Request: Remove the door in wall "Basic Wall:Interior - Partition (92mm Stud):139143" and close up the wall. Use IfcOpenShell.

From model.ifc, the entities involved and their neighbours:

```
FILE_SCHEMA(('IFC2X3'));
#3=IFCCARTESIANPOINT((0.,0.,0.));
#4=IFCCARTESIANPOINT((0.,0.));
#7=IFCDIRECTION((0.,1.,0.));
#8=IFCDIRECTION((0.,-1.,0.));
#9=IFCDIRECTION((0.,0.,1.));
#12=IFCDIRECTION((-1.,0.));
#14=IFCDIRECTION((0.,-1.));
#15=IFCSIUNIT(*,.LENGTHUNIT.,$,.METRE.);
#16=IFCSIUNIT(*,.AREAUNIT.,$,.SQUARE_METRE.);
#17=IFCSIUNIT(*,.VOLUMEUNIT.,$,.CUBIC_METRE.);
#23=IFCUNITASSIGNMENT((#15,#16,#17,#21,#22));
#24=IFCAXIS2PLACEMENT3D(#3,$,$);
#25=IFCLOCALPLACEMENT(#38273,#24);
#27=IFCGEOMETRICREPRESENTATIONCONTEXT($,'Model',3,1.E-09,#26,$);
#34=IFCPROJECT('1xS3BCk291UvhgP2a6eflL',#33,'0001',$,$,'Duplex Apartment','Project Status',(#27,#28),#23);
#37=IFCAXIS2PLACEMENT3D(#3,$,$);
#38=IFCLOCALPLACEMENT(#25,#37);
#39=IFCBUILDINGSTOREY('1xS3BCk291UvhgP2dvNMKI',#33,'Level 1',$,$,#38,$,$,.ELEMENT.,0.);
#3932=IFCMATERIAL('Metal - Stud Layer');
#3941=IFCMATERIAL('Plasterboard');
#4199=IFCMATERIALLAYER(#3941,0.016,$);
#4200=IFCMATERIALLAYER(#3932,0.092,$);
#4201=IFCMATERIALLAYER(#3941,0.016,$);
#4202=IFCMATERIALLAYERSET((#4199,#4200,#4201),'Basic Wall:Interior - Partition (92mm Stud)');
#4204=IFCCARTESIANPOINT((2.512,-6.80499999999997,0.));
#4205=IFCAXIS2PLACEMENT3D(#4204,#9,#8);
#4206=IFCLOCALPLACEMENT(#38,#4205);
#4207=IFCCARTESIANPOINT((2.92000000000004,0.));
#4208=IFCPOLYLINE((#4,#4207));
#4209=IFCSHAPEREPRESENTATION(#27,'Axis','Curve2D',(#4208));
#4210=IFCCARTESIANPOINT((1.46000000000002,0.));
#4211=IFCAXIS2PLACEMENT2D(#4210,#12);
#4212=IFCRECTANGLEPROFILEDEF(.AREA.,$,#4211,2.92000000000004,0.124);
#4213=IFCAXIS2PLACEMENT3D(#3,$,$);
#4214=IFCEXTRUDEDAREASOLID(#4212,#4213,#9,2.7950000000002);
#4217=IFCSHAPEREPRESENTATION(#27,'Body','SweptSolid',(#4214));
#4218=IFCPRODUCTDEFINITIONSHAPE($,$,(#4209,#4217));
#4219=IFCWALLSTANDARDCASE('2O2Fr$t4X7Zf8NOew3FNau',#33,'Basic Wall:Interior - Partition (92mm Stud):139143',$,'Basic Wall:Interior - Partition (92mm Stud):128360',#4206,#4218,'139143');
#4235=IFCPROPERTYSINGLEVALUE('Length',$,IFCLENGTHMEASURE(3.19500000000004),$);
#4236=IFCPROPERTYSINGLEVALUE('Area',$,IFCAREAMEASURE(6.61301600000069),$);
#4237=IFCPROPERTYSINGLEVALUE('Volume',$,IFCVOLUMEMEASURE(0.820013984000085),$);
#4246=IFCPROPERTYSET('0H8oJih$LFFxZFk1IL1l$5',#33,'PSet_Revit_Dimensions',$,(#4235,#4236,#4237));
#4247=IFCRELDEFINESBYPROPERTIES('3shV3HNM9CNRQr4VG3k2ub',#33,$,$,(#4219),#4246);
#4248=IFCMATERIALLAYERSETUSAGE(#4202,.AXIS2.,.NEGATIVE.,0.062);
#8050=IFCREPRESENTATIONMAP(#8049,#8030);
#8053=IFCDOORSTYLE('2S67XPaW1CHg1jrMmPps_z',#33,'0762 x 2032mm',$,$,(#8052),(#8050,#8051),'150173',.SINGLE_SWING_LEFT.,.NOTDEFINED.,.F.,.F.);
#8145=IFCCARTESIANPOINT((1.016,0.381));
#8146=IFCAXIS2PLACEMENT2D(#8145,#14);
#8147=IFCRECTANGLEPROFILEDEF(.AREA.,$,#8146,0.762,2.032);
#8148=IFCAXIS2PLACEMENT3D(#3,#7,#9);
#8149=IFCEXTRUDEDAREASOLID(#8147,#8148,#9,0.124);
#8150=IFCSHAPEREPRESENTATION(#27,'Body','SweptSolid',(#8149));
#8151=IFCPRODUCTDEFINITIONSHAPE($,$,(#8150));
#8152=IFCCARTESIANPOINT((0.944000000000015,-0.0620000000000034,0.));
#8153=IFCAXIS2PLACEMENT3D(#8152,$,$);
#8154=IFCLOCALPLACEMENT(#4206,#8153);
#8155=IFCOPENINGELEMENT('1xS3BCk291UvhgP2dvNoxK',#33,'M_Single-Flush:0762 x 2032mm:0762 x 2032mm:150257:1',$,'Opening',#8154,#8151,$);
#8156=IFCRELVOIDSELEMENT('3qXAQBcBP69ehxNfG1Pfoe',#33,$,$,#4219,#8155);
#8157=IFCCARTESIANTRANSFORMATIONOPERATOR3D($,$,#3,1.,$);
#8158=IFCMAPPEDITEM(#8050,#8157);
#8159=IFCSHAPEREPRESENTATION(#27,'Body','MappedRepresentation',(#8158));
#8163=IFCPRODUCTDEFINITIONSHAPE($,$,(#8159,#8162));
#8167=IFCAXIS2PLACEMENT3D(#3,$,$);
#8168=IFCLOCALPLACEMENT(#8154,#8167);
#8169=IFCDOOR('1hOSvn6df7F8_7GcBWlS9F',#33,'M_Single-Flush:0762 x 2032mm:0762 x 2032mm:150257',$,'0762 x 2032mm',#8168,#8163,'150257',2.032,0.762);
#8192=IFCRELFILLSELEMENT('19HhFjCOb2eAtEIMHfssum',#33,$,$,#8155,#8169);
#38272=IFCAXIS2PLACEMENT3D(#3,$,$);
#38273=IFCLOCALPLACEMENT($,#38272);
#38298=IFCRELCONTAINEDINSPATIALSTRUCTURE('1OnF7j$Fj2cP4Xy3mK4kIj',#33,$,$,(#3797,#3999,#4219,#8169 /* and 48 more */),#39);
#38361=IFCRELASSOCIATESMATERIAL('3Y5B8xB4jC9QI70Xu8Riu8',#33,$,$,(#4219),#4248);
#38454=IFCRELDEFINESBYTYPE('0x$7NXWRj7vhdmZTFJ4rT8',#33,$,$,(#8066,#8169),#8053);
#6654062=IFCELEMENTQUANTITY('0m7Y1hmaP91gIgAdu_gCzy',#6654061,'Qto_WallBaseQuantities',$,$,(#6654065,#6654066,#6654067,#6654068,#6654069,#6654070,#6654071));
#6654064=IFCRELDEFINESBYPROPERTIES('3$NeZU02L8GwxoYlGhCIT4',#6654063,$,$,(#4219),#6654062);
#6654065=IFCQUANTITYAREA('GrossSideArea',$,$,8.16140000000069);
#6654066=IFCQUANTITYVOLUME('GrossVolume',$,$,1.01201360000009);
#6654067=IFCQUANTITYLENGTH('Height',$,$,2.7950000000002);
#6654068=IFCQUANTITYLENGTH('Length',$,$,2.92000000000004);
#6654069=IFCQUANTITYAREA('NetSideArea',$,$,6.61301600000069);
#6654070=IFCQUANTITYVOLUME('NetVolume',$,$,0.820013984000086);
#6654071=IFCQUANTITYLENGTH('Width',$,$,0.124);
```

```python
import ifcopenshell
import ifcopenshell.api.feature
import ifcopenshell.api.pset
import ifcopenshell.api.root
import ifcopenshell.geom
import ifcopenshell.util.element
import ifcopenshell.util.shape
import ifcopenshell.util.unit

model = ifcopenshell.open("model.ifc")
area_scale = ifcopenshell.util.unit.calculate_unit_scale(model, "AREAUNIT")
volume_scale = ifcopenshell.util.unit.calculate_unit_scale(model, "VOLUMEUNIT")
settings = ifcopenshell.geom.settings()


def volume(element):
    """Net volume in cubic metres, openings subtracted."""
    shape = ifcopenshell.geom.create_shape(settings, element)
    return ifcopenshell.util.shape.get_volume(shape.geometry)


door = model.by_id(8169)
opening = door.FillsVoids[0].RelatingOpeningElement
wall = opening.VoidsElements[0].RelatingBuildingElement
before = volume(wall)

ifcopenshell.api.root.remove_product(model, product=door)
ifcopenshell.api.feature.remove_feature(model, feature=opening)

after = volume(wall)
thickness = 0.124  # wall thickness in metres

# Update the wall's stored quantities.
pset = model.by_id(ifcopenshell.util.element.get_pset(wall, "PSet_Revit_Dimensions", should_inherit=False)["id"])
ifcopenshell.api.pset.edit_pset(model, pset=pset, properties={
    "Area": model.create_entity("IfcAreaMeasure", after / thickness / area_scale),
    "Volume": model.create_entity("IfcVolumeMeasure", after / volume_scale),
})
qto = model.by_id(ifcopenshell.util.element.get_pset(wall, "Qto_WallBaseQuantities", should_inherit=False)["id"])
ifcopenshell.api.pset.edit_qto(model, qto=qto, properties={
    "NetSideArea": after / thickness / area_scale,
    "NetVolume": after / volume_scale,
})

print(f"wall volume {before:.3f} -> {after:.3f} m3")

model.write("model_rev.ifc")
```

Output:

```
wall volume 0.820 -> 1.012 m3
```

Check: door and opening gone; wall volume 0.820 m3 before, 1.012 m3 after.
